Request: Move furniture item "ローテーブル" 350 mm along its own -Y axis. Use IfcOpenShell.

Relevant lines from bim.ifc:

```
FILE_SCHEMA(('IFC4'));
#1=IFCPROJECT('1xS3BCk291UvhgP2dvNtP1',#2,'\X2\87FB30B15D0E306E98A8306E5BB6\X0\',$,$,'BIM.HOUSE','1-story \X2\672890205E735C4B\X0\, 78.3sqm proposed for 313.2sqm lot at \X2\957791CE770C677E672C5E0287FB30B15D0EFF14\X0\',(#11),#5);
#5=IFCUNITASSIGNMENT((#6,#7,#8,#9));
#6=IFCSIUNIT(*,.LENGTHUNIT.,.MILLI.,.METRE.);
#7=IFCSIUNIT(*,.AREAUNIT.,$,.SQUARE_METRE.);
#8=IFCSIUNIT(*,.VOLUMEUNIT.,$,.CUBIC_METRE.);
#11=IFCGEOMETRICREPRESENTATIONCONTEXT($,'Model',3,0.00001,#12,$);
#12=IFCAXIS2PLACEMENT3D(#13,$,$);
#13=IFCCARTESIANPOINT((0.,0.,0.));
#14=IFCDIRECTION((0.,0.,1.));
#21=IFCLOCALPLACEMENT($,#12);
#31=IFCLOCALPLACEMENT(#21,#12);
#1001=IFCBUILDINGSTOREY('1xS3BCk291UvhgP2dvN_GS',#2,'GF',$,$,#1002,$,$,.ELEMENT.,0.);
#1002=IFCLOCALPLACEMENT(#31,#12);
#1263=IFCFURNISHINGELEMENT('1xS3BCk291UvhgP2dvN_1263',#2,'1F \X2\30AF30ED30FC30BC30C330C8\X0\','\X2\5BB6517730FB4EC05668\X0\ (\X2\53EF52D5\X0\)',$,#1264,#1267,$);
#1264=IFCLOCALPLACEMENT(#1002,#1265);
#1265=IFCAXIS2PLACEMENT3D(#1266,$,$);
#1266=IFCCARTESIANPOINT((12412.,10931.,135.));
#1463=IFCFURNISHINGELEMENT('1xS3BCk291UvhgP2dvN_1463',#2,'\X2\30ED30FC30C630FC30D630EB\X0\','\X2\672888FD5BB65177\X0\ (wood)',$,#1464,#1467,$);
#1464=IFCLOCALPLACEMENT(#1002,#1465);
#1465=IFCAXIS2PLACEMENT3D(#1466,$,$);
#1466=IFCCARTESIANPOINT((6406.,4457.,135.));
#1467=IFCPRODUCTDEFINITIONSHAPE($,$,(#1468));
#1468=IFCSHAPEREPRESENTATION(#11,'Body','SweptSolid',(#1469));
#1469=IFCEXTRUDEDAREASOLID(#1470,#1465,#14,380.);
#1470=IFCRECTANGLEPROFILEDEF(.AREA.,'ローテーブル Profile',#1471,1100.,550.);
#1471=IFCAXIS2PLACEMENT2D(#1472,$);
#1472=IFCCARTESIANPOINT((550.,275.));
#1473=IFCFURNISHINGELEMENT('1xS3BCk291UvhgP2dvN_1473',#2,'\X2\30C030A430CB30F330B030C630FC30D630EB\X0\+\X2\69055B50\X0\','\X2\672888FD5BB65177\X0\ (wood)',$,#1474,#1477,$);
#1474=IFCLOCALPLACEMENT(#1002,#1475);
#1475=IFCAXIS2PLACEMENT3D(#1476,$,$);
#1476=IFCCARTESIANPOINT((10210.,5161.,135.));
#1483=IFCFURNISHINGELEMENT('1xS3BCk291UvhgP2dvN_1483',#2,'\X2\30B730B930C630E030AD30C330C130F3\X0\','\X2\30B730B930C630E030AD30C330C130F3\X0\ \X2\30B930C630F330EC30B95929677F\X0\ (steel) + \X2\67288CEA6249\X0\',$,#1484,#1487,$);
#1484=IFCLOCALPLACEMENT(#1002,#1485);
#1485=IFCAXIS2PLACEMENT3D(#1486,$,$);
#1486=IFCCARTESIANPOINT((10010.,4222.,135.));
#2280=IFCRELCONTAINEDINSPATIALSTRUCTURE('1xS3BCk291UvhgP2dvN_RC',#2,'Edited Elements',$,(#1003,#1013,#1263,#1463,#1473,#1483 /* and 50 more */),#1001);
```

```python
import ifcopenshell
import ifcopenshell.api.geometry
import ifcopenshell.util.placement

model = ifcopenshell.open("bim.ifc")

item = model.by_guid("1xS3BCk291UvhgP2dvN_1463")
matrix = ifcopenshell.util.placement.get_local_placement(item.ObjectPlacement)
matrix[:3, 3] -= matrix[:3, 1] * 350.0
ifcopenshell.api.geometry.edit_object_placement(model, product=item, matrix=matrix, is_si=False)

print(ifcopenshell.util.placement.get_local_placement(item.ObjectPlacement).round(3) + 0.0)

model.write("bim_rev.ifc")
```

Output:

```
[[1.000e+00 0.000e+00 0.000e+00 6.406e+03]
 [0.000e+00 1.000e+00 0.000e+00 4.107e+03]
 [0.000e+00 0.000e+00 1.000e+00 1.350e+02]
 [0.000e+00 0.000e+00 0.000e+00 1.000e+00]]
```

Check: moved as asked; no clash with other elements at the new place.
